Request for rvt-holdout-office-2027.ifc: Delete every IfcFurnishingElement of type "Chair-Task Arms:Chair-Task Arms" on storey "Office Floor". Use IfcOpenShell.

First a look at what the model holds.

```python
import ifcopenshell
import ifcopenshell.util.element

model = ifcopenshell.open("rvt-holdout-office-2027.ifc")
print(model.schema)
storey = next(s for s in model.by_type("IfcBuildingStorey") if s.Name == "Office Floor")
furniture = [e for e in ifcopenshell.util.element.get_decomposition(storey) if e.is_a("IfcFurnishingElement")]
seen = {}
for e in furniture:
    element_type = ifcopenshell.util.element.get_type(e)
    name = element_type.Name if element_type not in (None, e) else None
    seen[name] = seen.get(name, 0) + 1
for name, count in sorted(seen.items(), key=str):
    print(count, "x", name)
```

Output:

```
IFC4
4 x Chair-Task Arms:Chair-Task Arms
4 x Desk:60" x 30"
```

```python
import ifcopenshell
import ifcopenshell.api.root
import ifcopenshell.util.element

model = ifcopenshell.open("rvt-holdout-office-2027.ifc")

storey = next(s for s in model.by_type("IfcBuildingStorey") if s.Name == "Office Floor")
furniture = [e for e in ifcopenshell.util.element.get_decomposition(storey) if e.is_a("IfcFurnishingElement")]
targets = [e for e in furniture if (t := ifcopenshell.util.element.get_type(e)) not in (None, e) and t.Name == "Chair-Task Arms:Chair-Task Arms"]

for e in targets:
    ifcopenshell.api.root.remove_product(model, product=e)
print(len(targets), "removed")

model.write("rvt-holdout-office-2027_v2.ifc")
```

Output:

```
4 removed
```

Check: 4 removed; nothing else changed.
